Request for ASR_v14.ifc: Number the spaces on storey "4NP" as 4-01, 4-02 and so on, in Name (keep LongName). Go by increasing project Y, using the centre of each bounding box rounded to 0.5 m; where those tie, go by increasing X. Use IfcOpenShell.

First a look at what the model holds.

```python
import ifcopenshell
import ifcopenshell.util.element
import ifcopenshell.util.placement

model = ifcopenshell.open("ASR_v14.ifc")
print(model.schema)
storey = next(s for s in model.by_type("IfcBuildingStorey") if s.Name == "4NP")
spaces = [e for e in ifcopenshell.util.element.get_decomposition(storey) if e.is_a("IfcSpace")]
for e in sorted(spaces, key=lambda e: e.id()):
    origin = ifcopenshell.util.placement.get_local_placement(e.ObjectPlacement)[:3, 3]
    print(e.id(), e.Name, e.LongName, origin.round(2) + 0.0, sep=" | ")
```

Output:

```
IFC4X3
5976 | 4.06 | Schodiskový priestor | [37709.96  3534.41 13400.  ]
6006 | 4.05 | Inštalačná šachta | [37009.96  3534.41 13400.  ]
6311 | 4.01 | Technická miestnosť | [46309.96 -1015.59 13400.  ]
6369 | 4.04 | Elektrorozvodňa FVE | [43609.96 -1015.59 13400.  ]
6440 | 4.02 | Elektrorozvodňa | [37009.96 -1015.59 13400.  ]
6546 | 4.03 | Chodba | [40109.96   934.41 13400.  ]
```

```python
import ifcopenshell
import ifcopenshell.geom
import ifcopenshell.util.element
import ifcopenshell.util.shape

model = ifcopenshell.open("ASR_v14.ifc")
settings = ifcopenshell.geom.settings()
settings.set("use-world-coords", True)


def centre(element):
    shape = ifcopenshell.geom.create_shape(settings, element)
    return ifcopenshell.util.shape.get_bbox_centroid(shape.geometry)


storey = next(s for s in model.by_type("IfcBuildingStorey") if s.Name == "4NP")
spaces = [e for e in ifcopenshell.util.element.get_decomposition(storey) if e.is_a("IfcSpace")]

# Insertion points can sit at a corner or the storey origin, so sort by the geometry (in metres).
centres = {e: centre(e) for e in spaces}
spaces.sort(key=lambda e: (round(centres[e][1] / 0.5), centres[e][0]))

for i, e in enumerate(spaces, start=1):
    number = f"4-{i:02d}"
    e.Name = number
    print(e.id(), number)

model.write("ASR_v14-out.ifc")
```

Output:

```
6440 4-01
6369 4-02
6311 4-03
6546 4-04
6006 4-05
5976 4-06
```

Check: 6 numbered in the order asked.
